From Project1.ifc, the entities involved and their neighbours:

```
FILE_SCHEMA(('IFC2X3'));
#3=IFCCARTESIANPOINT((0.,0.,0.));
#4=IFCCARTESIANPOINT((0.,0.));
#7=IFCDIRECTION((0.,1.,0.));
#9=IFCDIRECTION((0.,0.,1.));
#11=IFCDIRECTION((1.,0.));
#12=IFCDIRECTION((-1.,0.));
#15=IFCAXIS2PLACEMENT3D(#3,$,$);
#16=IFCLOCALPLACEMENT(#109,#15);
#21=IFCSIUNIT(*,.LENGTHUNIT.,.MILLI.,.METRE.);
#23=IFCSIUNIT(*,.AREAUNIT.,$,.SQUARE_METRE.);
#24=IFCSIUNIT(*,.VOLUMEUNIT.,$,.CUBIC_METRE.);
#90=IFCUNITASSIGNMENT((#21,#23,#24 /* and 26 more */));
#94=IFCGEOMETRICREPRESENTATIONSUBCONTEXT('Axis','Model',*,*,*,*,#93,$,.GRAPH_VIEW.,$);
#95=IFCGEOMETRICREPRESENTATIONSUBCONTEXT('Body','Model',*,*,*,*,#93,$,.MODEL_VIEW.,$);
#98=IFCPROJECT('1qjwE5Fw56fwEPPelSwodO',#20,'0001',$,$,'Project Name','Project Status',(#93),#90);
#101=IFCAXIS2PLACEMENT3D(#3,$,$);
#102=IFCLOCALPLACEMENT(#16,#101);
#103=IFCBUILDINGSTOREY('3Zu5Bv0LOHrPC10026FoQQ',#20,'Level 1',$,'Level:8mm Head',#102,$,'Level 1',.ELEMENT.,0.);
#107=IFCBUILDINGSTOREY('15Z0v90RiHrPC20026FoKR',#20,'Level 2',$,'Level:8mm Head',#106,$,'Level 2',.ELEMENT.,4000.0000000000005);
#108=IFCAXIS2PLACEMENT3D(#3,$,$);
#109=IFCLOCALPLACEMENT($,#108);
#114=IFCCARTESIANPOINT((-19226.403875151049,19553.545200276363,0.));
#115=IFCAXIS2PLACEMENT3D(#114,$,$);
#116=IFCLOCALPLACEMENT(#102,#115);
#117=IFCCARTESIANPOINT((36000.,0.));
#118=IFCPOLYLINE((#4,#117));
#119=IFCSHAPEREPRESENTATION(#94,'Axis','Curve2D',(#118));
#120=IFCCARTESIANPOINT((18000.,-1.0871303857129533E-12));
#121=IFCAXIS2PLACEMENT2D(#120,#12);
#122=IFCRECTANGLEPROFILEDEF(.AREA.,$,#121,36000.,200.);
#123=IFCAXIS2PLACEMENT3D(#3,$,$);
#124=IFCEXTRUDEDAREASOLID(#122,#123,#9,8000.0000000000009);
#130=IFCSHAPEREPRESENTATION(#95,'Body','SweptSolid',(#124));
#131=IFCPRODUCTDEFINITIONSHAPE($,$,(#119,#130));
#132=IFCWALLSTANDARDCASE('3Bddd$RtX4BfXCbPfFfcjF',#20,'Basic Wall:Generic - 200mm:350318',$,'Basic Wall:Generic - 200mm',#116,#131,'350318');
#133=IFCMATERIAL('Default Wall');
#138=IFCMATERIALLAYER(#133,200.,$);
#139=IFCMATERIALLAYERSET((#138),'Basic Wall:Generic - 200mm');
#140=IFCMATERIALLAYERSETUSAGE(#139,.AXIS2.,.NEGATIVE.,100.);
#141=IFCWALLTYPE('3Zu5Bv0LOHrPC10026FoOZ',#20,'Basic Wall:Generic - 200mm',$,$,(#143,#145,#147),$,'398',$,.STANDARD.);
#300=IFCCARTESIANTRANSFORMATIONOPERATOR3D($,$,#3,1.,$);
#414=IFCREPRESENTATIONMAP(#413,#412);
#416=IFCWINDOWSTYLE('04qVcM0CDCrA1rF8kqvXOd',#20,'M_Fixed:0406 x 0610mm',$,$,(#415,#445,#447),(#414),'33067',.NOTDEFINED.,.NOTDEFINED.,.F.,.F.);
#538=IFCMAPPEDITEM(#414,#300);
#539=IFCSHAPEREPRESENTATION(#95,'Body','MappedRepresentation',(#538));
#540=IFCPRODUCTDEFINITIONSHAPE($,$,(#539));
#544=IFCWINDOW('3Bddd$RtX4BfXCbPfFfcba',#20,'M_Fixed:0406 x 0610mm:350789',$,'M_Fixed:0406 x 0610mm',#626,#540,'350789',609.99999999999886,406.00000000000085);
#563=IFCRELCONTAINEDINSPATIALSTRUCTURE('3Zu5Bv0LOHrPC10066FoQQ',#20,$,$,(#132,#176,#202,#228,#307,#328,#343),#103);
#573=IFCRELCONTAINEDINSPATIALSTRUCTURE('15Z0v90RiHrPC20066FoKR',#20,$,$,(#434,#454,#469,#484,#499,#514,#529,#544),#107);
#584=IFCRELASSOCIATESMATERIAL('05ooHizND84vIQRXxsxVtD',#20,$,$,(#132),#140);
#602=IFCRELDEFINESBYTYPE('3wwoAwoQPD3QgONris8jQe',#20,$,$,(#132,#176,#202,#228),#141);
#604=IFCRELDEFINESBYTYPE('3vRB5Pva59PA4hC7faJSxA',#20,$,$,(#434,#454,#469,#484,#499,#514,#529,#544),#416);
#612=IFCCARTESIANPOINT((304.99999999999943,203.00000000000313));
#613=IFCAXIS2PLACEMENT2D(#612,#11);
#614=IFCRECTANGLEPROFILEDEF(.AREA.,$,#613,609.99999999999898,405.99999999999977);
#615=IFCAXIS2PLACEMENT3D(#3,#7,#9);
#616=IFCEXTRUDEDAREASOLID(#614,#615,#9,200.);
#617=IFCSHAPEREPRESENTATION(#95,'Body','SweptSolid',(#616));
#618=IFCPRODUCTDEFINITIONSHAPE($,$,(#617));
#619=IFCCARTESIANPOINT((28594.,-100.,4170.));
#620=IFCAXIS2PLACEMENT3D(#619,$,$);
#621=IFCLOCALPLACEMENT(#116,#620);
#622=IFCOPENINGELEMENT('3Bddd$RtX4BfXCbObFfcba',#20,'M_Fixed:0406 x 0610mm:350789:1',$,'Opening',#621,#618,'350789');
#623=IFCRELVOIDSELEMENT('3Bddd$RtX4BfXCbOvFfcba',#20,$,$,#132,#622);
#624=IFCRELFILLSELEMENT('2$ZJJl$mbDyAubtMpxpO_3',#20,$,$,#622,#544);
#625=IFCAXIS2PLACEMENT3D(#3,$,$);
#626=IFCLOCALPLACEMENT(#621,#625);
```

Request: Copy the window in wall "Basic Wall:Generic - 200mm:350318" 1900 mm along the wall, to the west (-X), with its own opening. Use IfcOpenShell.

```python
import ifcopenshell
import ifcopenshell.api.feature
import ifcopenshell.api.geometry
import ifcopenshell.api.root
import ifcopenshell.geom
import ifcopenshell.util.element
import ifcopenshell.util.placement
import ifcopenshell.util.shape

model = ifcopenshell.open("Project1.ifc")
settings = ifcopenshell.geom.settings()


def volume(element):
    """Net volume in cubic metres, openings subtracted."""
    shape = ifcopenshell.geom.create_shape(settings, element)
    return ifcopenshell.util.shape.get_volume(shape.geometry)


def reuse_history(source, copy):
    """copy_class also copies each property set's owner history, people and application; keep the originals."""
    for rel in copy.IsDefinedBy:
        if rel.is_a("IfcRelDefinesByProperties") and (history := rel.RelatingPropertyDefinition.OwnerHistory):
            rel.RelatingPropertyDefinition.OwnerHistory = source.OwnerHistory
            ifcopenshell.util.element.remove_deep2(model, history)


window = model.by_guid("3Bddd$RtX4BfXCbPfFfcba")
opening = window.FillsVoids[0].RelatingOpeningElement
wall = opening.VoidsElements[0].RelatingBuildingElement
before = volume(wall)
shift = ifcopenshell.util.placement.get_local_placement(wall.ObjectPlacement)[:3, 0] * -1900.0

# copy_class copies the void relationship, type, container and properties, but no geometry.
new_opening = ifcopenshell.api.root.copy_class(model, product=opening)
new_opening.Representation = ifcopenshell.util.element.copy_deep(
    model, opening.Representation, exclude=["IfcGeometricRepresentationContext", "IfcRepresentationMap"]
)
new_opening.Name = "M_Fixed:0406 x 0610mm"
new_opening.Tag = None
new_window = ifcopenshell.api.root.copy_class(model, product=window)
new_window.Representation = ifcopenshell.util.element.copy_deep(
    model, window.Representation, exclude=["IfcGeometricRepresentationContext", "IfcRepresentationMap"]
)
new_window.Name = "M_Fixed:0406 x 0610mm"
new_window.Tag = None
reuse_history(window, new_window)
fills = ifcopenshell.api.feature.add_filling(model, opening=new_opening, element=new_window)
fills.OwnerHistory = new_window.OwnerHistory  # required in IFC2X3

for old, new in ((opening, new_opening), (window, new_window)):
    matrix = ifcopenshell.util.placement.get_local_placement(old.ObjectPlacement)
    matrix[:3, 3] += shift
    ifcopenshell.api.geometry.edit_object_placement(model, product=new, matrix=matrix, is_si=False)

after = volume(wall)

print(f"wall volume {before:.3f} -> {after:.3f} m3")

model.write("Project1-out.ifc")
```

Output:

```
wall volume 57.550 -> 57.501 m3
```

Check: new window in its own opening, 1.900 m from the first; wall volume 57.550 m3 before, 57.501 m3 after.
